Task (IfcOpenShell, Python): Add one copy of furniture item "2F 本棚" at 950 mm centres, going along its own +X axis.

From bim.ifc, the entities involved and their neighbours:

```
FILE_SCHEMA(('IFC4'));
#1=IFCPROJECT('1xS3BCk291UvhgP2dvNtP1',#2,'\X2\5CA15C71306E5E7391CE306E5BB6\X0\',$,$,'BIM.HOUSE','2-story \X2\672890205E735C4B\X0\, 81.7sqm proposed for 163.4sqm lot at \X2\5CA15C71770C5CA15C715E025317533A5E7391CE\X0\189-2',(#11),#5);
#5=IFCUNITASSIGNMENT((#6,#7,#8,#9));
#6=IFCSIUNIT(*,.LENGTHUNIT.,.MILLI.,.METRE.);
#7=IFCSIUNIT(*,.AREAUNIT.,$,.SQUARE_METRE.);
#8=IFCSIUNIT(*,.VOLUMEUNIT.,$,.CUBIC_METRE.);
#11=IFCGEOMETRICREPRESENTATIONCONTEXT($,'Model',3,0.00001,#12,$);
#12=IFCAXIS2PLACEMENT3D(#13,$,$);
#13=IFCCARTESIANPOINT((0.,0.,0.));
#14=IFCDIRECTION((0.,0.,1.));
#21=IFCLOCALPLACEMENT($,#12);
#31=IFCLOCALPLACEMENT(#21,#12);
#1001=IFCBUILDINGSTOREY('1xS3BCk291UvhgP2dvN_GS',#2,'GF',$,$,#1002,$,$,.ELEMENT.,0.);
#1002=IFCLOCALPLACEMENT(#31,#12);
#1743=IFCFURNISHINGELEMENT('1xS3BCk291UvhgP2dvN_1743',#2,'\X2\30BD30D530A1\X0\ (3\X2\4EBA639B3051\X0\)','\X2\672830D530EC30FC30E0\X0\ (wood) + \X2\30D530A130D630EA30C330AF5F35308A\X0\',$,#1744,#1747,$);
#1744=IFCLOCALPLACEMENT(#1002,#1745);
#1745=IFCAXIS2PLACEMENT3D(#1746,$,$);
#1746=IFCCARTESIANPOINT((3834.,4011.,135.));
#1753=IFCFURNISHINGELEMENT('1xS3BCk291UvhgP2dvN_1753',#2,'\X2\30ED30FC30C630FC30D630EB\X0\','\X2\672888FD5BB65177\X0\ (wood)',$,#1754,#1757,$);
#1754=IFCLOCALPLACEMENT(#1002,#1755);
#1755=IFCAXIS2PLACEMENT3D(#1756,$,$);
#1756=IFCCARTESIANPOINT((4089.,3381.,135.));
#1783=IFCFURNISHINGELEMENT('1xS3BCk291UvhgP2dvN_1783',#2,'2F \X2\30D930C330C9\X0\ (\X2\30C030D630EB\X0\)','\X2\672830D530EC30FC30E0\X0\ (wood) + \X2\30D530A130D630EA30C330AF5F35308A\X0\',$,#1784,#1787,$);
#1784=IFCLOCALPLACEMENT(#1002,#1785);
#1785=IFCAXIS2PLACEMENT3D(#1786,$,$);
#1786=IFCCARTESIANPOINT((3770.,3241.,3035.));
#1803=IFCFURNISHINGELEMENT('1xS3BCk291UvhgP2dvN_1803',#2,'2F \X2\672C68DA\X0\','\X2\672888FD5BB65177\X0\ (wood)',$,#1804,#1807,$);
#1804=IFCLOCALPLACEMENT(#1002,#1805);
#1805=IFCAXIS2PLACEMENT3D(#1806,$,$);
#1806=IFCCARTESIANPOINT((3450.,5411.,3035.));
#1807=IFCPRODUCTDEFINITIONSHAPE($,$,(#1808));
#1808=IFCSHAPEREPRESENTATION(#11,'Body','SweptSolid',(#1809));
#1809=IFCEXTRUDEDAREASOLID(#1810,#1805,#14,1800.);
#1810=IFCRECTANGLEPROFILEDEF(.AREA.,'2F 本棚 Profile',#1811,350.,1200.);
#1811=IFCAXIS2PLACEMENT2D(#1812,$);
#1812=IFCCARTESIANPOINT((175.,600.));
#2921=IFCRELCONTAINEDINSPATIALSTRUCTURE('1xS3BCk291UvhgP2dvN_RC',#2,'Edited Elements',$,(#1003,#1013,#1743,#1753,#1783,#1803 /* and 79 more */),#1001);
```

```python
import ifcopenshell
import ifcopenshell.api.geometry
import ifcopenshell.api.root
import ifcopenshell.util.element
import ifcopenshell.util.placement

model = ifcopenshell.open("bim.ifc")


def reuse_history(source, copy):
    """copy_class also copies each property set's owner history, people and application; keep the originals."""
    for rel in copy.IsDefinedBy:
        if rel.is_a("IfcRelDefinesByProperties") and (history := rel.RelatingPropertyDefinition.OwnerHistory):
            rel.RelatingPropertyDefinition.OwnerHistory = source.OwnerHistory
            ifcopenshell.util.element.remove_deep2(model, history)


source = model.by_guid("1xS3BCk291UvhgP2dvN_1803")
base = ifcopenshell.util.placement.get_local_placement(source.ObjectPlacement)
step = base[:3, 0] * 950.0

for i in range(1, 2):
    copy = ifcopenshell.api.root.copy_class(model, product=source)
    copy.Representation = ifcopenshell.util.element.copy_deep(
        model, source.Representation, exclude=["IfcGeometricRepresentationContext", "IfcRepresentationMap"]
    )
    reuse_history(source, copy)
    matrix = base.copy()
    matrix[:3, 3] += i * step
    print("added at", matrix[:3, 3].round(3) + 0.0)
    ifcopenshell.api.geometry.edit_object_placement(model, product=copy, matrix=matrix, is_si=False)

model.write("bim_edited.ifc")
```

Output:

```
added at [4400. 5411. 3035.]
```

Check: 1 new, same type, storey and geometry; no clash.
